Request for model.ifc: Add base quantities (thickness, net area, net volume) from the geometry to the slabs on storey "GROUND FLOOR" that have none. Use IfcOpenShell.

First a look at what the model holds.

```python
import ifcopenshell
import ifcopenshell.util.element
import ifcopenshell.util.unit

model = ifcopenshell.open("model.ifc")
print(model.schema)
for unit_type in ("LENGTHUNIT", "AREAUNIT", "VOLUMEUNIT"):
    print(unit_type, ifcopenshell.util.unit.calculate_unit_scale(model, unit_type))
storey = next(s for s in model.by_type("IfcBuildingStorey") if s.Name == "GROUND FLOOR")
slabs = [e for e in ifcopenshell.util.element.get_decomposition(storey) if e.is_a("IfcSlab")]
for e in sorted(slabs, key=lambda e: e.id()):
    print(e.id(), e.is_a(), e.Name, list(ifcopenshell.util.element.get_psets(e, qtos_only=True)), sep=" | ")
```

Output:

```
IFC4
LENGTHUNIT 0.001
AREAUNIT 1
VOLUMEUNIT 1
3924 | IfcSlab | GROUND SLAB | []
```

```python
import ifcopenshell
import ifcopenshell.api.pset
import ifcopenshell.geom
import ifcopenshell.util.element
import ifcopenshell.util.shape
import ifcopenshell.util.unit

model = ifcopenshell.open("model.ifc")
unit_scale = ifcopenshell.util.unit.calculate_unit_scale(model)
area_scale = ifcopenshell.util.unit.calculate_unit_scale(model, "AREAUNIT")
volume_scale = ifcopenshell.util.unit.calculate_unit_scale(model, "VOLUMEUNIT")
settings = ifcopenshell.geom.settings()

storey = next(s for s in model.by_type("IfcBuildingStorey") if s.Name == "GROUND FLOOR")
slabs = [e for e in ifcopenshell.util.element.get_decomposition(storey) if e.is_a("IfcSlab")]

for e in sorted(slabs, key=lambda e: e.id()):
    if ifcopenshell.util.element.get_psets(e, qtos_only=True, should_inherit=False):
        continue
    # Geometry comes back in metres, in the element's own axes.
    shape = ifcopenshell.geom.create_shape(settings, e)
    values = {
        "Width": ifcopenshell.util.shape.get_z(shape.geometry) / unit_scale,
        "NetArea": ifcopenshell.util.shape.get_footprint_area(shape.geometry) / area_scale,
        "NetVolume": ifcopenshell.util.shape.get_volume(shape.geometry) / volume_scale,
    }
    qto = ifcopenshell.api.pset.add_qto(model, product=e, name="Qto_SlabBaseQuantities")
    ifcopenshell.api.pset.edit_qto(model, qto=qto, properties=values)
    print(e.id(), {k: round(v, 3) for k, v in values.items()})

model.write("model_updated.ifc")
```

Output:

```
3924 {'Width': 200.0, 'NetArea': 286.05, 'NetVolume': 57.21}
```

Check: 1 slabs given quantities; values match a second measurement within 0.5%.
